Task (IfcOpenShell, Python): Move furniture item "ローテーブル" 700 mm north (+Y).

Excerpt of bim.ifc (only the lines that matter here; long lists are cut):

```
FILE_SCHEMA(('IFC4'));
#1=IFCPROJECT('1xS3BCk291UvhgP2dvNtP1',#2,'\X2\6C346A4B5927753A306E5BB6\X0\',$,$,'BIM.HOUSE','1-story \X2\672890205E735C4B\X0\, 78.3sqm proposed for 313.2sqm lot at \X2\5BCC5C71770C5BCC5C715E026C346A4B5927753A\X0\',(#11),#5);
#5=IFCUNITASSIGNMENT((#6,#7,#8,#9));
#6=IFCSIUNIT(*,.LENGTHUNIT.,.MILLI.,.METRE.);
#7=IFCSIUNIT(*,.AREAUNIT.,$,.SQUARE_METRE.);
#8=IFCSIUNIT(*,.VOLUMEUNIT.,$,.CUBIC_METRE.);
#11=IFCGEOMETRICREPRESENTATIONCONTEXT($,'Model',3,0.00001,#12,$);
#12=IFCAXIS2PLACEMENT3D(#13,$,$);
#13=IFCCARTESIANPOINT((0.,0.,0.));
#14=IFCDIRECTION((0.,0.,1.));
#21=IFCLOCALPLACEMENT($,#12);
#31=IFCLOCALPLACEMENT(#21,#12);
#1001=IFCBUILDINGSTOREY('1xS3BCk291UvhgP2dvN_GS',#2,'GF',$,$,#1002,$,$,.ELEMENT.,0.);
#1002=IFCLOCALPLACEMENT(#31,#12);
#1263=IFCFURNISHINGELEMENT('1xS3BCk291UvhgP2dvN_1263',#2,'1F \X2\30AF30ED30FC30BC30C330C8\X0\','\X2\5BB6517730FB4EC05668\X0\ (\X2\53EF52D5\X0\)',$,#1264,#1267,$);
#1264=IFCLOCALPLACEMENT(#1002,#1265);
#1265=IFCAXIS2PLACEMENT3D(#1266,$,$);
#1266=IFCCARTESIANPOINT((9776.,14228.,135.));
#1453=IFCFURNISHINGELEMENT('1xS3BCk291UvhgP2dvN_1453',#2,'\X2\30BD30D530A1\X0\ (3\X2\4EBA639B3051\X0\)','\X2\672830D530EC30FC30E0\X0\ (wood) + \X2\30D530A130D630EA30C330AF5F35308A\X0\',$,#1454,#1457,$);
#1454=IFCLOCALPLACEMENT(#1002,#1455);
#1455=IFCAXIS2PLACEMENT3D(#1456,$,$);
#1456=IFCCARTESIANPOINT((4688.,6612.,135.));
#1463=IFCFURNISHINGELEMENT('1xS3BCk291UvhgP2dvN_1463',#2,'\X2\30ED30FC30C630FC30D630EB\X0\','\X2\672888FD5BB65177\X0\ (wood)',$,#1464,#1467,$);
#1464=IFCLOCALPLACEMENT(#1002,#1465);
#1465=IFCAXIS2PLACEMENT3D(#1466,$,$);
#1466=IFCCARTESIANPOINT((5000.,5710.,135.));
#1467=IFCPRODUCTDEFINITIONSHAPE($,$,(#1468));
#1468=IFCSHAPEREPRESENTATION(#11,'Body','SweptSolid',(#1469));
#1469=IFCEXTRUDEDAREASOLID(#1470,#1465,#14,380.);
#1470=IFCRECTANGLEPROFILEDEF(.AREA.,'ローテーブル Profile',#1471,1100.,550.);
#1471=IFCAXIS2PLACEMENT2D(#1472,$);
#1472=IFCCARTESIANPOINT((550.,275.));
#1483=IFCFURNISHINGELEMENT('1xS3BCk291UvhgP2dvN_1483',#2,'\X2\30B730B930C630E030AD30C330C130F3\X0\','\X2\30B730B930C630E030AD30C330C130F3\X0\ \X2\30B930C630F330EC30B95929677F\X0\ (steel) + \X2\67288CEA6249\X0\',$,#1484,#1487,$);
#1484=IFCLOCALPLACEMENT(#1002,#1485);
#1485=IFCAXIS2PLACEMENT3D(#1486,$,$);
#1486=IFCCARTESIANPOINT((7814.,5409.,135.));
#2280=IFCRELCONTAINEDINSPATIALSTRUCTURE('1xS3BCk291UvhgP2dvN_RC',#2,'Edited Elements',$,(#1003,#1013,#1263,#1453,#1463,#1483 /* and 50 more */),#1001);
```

```python
import ifcopenshell
import ifcopenshell.api.geometry
import ifcopenshell.util.placement
import ifcopenshell.util.unit

model = ifcopenshell.open("bim.ifc")
unit_scale = ifcopenshell.util.unit.calculate_unit_scale(model)

item = model.by_guid("1xS3BCk291UvhgP2dvN_1463")
matrix = ifcopenshell.util.placement.get_local_placement(item.ObjectPlacement)
matrix[1, 3] += 0.7 / unit_scale
ifcopenshell.api.geometry.edit_object_placement(model, product=item, matrix=matrix, is_si=False)

print(ifcopenshell.util.placement.get_local_placement(item.ObjectPlacement).round(3) + 0.0)

model.write("bim_edited.ifc")
```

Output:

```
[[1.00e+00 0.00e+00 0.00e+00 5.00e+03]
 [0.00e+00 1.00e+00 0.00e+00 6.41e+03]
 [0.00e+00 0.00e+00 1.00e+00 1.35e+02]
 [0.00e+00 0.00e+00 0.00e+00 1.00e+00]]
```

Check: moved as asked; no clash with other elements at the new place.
